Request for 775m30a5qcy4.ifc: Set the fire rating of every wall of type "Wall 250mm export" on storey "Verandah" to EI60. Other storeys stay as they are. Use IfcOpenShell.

First a look at what the model holds.

```python
import ifcopenshell
import ifcopenshell.util.element

model = ifcopenshell.open("775m30a5qcy4.ifc")
print(model.schema)
storey = next(s for s in model.by_type("IfcBuildingStorey") if s.Name == "Verandah")
walls = [e for e in ifcopenshell.util.element.get_decomposition(storey) if e.is_a("IfcWall")]
seen = {}
for e in walls:
    element_type = ifcopenshell.util.element.get_type(e)
    key = (element_type.Name if element_type != e and element_type else None, ifcopenshell.util.element.get_pset(e, "Pset_WallCommon", "FireRating"))
    seen[key] = seen.get(key, 0) + 1
for (name, value), count in sorted(seen.items(), key=str):
    print(count, "x", name, "|", value)
```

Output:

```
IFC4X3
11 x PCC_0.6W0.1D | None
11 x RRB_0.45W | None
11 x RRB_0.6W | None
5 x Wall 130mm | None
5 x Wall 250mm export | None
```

```python
import ifcopenshell
import ifcopenshell.api.pset
import ifcopenshell.util.element

model = ifcopenshell.open("775m30a5qcy4.ifc")

storey = next(s for s in model.by_type("IfcBuildingStorey") if s.Name == "Verandah")
walls = [e for e in ifcopenshell.util.element.get_decomposition(storey) if e.is_a("IfcWall")]

count = 0
for e in walls:
    element_type = ifcopenshell.util.element.get_type(e)
    if element_type in (None, e) or element_type.Name != "Wall 250mm export":
        continue
    # add_pset returns the element's existing set when there is one.
    pset = ifcopenshell.api.pset.add_pset(model, product=e, name="Pset_WallCommon")
    ifcopenshell.api.pset.edit_pset(model, pset=pset, properties={"FireRating": "EI60"})
    count += 1

print(count, "walls updated")

model.write("775m30a5qcy4-out.ifc")
```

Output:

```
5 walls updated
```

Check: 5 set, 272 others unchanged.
